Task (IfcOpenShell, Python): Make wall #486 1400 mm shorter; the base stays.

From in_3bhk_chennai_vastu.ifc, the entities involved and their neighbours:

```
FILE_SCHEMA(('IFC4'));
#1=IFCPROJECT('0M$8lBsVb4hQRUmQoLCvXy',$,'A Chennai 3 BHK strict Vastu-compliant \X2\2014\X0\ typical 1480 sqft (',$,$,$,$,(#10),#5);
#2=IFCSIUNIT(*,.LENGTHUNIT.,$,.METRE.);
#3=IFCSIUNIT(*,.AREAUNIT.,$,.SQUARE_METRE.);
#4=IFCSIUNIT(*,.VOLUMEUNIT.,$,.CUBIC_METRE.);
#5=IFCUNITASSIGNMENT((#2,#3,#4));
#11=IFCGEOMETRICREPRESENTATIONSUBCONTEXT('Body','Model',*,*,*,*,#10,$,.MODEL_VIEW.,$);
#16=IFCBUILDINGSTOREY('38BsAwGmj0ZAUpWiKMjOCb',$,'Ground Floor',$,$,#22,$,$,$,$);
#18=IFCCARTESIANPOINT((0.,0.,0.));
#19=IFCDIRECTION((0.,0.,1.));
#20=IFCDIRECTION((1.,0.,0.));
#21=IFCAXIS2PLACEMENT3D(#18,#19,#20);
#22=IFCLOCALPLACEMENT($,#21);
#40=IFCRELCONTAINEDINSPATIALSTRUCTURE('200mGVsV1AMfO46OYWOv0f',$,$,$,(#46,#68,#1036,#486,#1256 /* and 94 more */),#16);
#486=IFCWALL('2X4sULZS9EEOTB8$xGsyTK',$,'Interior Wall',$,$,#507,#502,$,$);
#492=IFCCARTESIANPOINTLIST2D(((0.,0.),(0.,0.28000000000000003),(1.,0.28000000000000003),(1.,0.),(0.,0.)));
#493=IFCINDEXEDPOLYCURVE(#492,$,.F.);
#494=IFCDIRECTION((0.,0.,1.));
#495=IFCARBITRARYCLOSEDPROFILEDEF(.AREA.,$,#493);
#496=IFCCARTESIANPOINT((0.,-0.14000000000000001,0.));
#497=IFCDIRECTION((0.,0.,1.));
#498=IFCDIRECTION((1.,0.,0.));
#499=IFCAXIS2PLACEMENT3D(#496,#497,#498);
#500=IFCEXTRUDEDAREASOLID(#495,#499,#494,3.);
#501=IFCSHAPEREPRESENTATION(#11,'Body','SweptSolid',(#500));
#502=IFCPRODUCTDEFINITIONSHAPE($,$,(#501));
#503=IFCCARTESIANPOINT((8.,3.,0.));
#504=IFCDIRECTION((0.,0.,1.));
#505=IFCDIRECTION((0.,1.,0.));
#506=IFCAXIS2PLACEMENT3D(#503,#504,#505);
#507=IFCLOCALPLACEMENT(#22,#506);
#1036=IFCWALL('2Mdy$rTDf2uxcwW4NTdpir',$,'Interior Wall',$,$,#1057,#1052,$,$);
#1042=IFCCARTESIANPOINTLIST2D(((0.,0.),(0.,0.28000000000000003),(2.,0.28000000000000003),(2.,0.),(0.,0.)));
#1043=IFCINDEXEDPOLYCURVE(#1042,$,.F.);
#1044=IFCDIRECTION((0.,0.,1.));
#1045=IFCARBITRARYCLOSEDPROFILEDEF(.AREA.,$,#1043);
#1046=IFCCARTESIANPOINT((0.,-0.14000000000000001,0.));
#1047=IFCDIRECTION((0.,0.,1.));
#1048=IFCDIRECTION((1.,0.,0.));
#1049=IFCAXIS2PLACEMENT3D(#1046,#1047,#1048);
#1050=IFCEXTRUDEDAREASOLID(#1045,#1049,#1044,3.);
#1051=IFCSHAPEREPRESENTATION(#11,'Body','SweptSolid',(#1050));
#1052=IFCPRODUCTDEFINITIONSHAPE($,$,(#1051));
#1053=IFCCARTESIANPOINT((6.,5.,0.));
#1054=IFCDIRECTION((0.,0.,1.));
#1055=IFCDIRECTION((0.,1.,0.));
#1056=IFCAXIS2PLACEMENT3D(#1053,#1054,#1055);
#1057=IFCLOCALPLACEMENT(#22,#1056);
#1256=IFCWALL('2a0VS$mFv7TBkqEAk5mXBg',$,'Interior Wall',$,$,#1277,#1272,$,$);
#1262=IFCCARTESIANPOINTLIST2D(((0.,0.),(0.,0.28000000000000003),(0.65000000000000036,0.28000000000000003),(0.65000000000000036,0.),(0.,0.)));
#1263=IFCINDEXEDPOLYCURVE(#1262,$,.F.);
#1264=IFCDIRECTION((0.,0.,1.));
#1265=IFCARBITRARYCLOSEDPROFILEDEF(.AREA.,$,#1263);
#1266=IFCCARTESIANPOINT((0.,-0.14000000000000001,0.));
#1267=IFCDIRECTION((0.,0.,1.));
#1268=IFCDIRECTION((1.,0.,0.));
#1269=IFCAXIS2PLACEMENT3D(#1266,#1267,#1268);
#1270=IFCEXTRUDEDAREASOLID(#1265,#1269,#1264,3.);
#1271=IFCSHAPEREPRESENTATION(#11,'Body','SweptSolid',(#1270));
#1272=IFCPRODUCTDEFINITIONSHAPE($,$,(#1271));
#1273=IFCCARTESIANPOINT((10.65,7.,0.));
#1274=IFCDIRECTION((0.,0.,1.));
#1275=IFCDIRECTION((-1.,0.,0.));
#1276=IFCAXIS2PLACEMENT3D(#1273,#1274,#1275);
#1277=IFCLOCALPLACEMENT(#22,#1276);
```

```python
import ifcopenshell
import ifcopenshell.geom
import ifcopenshell.util.representation
import ifcopenshell.util.shape
import ifcopenshell.util.unit

model = ifcopenshell.open("in_3bhk_chennai_vastu.ifc")
unit_scale = ifcopenshell.util.unit.calculate_unit_scale(model)
settings = ifcopenshell.geom.settings()


def volume(element):
    """Net volume in cubic metres, openings subtracted."""
    shape = ifcopenshell.geom.create_shape(settings, element)
    return ifcopenshell.util.shape.get_volume(shape.geometry)


wall = model.by_guid("2X4sULZS9EEOTB8$xGsyTK")
before = volume(wall)

body = ifcopenshell.util.representation.get_representation(wall, "Model", "Body")
solid = body.Items[0]
old_height = solid.Depth
solid.Depth -= 1.4 / unit_scale
after = volume(wall)

print(f"height {old_height:g} -> {solid.Depth:g}, volume {before:.3f} -> {after:.3f} m3")

model.write("in_3bhk_chennai_vastu_edited.ifc")
```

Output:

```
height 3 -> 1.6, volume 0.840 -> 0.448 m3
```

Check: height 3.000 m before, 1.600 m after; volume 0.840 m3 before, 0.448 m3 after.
